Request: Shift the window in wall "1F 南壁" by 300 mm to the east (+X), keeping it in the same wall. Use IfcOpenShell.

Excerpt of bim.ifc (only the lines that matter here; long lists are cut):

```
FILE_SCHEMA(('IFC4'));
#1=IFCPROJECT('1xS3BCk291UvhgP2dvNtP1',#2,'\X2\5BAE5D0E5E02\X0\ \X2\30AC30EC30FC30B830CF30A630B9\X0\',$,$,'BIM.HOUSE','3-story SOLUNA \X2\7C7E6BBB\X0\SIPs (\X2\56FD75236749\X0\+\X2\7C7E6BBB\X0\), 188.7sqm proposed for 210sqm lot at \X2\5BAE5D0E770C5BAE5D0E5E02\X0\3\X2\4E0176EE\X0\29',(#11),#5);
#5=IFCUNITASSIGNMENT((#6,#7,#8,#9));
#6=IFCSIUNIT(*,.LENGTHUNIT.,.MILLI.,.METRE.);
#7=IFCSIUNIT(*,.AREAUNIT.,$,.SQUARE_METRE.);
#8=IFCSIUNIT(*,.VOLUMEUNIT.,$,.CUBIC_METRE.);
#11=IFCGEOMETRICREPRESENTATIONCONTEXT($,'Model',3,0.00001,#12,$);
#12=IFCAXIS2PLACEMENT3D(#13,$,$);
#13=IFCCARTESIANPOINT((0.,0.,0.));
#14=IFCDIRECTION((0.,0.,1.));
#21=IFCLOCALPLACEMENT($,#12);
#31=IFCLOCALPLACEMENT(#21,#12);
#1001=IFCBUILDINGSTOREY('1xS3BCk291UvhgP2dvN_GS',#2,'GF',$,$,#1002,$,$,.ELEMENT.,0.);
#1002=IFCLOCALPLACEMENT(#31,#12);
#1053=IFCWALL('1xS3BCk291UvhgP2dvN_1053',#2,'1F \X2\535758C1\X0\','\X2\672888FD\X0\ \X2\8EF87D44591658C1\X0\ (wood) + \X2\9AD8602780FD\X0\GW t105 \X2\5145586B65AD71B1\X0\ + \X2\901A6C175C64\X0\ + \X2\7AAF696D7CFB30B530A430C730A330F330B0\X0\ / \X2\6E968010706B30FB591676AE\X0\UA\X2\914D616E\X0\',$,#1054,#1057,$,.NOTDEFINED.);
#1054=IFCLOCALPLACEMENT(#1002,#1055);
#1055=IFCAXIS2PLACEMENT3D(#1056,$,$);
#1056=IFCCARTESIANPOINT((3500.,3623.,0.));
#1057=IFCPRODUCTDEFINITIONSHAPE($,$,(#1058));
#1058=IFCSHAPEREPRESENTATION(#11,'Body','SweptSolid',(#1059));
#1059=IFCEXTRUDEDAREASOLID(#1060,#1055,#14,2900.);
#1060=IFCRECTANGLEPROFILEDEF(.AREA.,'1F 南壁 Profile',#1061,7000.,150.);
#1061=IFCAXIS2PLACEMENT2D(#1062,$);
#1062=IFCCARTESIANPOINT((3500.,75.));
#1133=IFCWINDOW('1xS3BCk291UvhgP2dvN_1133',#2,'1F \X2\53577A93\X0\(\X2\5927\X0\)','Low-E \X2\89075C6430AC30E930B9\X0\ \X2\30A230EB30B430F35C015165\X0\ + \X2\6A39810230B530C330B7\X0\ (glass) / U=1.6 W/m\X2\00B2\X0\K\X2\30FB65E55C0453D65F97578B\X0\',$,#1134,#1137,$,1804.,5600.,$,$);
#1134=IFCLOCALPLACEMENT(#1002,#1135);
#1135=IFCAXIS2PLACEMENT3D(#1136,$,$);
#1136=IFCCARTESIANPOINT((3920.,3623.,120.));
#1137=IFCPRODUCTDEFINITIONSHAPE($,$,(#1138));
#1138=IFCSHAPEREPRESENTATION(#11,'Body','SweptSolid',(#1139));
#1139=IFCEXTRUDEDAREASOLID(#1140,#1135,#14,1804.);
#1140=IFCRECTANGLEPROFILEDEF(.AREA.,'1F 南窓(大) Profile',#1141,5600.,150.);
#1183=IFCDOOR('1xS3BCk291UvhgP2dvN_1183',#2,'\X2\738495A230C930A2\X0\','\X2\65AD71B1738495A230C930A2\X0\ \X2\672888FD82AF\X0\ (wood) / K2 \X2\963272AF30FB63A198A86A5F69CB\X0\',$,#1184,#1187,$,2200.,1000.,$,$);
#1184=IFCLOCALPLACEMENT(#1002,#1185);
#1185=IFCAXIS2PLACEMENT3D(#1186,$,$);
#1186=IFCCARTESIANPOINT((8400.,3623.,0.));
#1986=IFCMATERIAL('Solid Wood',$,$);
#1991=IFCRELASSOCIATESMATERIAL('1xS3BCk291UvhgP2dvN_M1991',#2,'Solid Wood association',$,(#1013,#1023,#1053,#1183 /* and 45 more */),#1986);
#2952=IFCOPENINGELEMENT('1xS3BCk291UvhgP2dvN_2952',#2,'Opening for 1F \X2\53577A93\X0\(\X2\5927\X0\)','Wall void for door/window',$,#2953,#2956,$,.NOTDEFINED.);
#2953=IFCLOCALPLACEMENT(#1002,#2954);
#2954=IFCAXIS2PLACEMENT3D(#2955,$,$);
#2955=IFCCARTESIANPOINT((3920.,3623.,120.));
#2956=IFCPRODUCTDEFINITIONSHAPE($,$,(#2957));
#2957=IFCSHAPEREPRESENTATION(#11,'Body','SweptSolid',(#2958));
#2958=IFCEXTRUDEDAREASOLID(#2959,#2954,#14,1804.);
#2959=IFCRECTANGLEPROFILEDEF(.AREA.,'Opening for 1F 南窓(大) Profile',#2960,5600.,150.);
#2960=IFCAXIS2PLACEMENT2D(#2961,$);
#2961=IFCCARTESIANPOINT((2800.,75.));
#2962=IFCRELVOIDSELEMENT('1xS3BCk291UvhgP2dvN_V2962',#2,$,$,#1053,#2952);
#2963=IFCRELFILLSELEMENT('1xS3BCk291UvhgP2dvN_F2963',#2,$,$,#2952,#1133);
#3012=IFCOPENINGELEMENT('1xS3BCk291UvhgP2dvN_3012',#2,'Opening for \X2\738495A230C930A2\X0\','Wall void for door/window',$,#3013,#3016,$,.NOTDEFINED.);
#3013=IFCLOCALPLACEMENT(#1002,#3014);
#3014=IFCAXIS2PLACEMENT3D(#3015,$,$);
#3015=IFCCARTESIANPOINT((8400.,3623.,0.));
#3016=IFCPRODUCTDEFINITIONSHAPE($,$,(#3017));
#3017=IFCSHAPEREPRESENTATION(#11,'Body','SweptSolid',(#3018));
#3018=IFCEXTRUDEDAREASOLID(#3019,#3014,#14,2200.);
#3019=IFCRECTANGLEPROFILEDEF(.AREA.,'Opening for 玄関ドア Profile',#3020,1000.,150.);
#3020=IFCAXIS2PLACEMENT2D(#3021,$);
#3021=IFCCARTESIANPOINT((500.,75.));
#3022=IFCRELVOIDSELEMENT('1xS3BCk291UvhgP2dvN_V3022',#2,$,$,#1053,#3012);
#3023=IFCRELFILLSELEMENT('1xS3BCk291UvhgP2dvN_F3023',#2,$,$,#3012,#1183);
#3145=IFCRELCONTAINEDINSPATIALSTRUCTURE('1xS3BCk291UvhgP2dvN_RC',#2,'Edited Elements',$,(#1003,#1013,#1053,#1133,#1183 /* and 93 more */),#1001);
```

```python
import ifcopenshell
import ifcopenshell.api.geometry
import ifcopenshell.util.placement

model = ifcopenshell.open("bim.ifc")

window = model.by_guid("1xS3BCk291UvhgP2dvN_1133")
opening = window.FillsVoids[0].RelatingOpeningElement
wall = opening.VoidsElements[0].RelatingBuildingElement

wall_matrix = ifcopenshell.util.placement.get_local_placement(wall.ObjectPlacement)
shift = wall_matrix[:3, 0] * 300.0
before = ifcopenshell.util.placement.get_local_placement(window.ObjectPlacement)[:3, 3].copy()

# The window is not placed relative to its opening, so move both.
for product in (opening, window):
    matrix = ifcopenshell.util.placement.get_local_placement(product.ObjectPlacement)
    matrix[:3, 3] += shift
    ifcopenshell.api.geometry.edit_object_placement(model, product=product, matrix=matrix, is_si=False)

after = ifcopenshell.util.placement.get_local_placement(window.ObjectPlacement)[:3, 3]
print("window moved by", (after - before).round(3) + 0.0)

model.write("bim_updated.ifc")
```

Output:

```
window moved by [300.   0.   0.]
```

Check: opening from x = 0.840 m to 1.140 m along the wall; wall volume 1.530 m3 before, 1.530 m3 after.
